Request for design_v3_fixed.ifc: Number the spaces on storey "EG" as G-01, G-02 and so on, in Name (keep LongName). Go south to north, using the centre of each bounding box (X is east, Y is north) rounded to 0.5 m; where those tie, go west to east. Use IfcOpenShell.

First a look at what the model holds.

```python
import ifcopenshell
import ifcopenshell.util.element
import ifcopenshell.util.placement

model = ifcopenshell.open("design_v3_fixed.ifc")
print(model.schema)
storey = next(s for s in model.by_type("IfcBuildingStorey") if s.Name == "EG")
spaces = [e for e in ifcopenshell.util.element.get_decomposition(storey) if e.is_a("IfcSpace")]
for e in sorted(spaces, key=lambda e: e.id()):
    origin = ifcopenshell.util.placement.get_local_placement(e.ObjectPlacement)[:3, 3]
    print(e.id(), e.Name, e.LongName, origin.round(2) + 0.0, sep=" | ")
```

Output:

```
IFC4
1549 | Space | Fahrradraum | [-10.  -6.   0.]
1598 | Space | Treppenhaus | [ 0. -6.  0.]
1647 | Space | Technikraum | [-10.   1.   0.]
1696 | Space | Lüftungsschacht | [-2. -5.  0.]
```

```python
import ifcopenshell
import ifcopenshell.geom
import ifcopenshell.util.element
import ifcopenshell.util.shape

model = ifcopenshell.open("design_v3_fixed.ifc")
settings = ifcopenshell.geom.settings()
settings.set("use-world-coords", True)


def centre(element):
    shape = ifcopenshell.geom.create_shape(settings, element)
    return ifcopenshell.util.shape.get_bbox_centroid(shape.geometry)


storey = next(s for s in model.by_type("IfcBuildingStorey") if s.Name == "EG")
spaces = [e for e in ifcopenshell.util.element.get_decomposition(storey) if e.is_a("IfcSpace")]

# Insertion points can sit at a corner or the storey origin, so sort by the geometry (in metres).
centres = {e: centre(e) for e in spaces}
spaces.sort(key=lambda e: (round(centres[e][1] / 0.5), centres[e][0]))

for i, e in enumerate(spaces, start=1):
    number = f"G-{i:02d}"
    e.Name = number
    print(e.id(), number)

model.write("design_v3_fixed-out.ifc")
```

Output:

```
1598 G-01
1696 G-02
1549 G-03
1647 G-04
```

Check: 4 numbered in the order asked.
